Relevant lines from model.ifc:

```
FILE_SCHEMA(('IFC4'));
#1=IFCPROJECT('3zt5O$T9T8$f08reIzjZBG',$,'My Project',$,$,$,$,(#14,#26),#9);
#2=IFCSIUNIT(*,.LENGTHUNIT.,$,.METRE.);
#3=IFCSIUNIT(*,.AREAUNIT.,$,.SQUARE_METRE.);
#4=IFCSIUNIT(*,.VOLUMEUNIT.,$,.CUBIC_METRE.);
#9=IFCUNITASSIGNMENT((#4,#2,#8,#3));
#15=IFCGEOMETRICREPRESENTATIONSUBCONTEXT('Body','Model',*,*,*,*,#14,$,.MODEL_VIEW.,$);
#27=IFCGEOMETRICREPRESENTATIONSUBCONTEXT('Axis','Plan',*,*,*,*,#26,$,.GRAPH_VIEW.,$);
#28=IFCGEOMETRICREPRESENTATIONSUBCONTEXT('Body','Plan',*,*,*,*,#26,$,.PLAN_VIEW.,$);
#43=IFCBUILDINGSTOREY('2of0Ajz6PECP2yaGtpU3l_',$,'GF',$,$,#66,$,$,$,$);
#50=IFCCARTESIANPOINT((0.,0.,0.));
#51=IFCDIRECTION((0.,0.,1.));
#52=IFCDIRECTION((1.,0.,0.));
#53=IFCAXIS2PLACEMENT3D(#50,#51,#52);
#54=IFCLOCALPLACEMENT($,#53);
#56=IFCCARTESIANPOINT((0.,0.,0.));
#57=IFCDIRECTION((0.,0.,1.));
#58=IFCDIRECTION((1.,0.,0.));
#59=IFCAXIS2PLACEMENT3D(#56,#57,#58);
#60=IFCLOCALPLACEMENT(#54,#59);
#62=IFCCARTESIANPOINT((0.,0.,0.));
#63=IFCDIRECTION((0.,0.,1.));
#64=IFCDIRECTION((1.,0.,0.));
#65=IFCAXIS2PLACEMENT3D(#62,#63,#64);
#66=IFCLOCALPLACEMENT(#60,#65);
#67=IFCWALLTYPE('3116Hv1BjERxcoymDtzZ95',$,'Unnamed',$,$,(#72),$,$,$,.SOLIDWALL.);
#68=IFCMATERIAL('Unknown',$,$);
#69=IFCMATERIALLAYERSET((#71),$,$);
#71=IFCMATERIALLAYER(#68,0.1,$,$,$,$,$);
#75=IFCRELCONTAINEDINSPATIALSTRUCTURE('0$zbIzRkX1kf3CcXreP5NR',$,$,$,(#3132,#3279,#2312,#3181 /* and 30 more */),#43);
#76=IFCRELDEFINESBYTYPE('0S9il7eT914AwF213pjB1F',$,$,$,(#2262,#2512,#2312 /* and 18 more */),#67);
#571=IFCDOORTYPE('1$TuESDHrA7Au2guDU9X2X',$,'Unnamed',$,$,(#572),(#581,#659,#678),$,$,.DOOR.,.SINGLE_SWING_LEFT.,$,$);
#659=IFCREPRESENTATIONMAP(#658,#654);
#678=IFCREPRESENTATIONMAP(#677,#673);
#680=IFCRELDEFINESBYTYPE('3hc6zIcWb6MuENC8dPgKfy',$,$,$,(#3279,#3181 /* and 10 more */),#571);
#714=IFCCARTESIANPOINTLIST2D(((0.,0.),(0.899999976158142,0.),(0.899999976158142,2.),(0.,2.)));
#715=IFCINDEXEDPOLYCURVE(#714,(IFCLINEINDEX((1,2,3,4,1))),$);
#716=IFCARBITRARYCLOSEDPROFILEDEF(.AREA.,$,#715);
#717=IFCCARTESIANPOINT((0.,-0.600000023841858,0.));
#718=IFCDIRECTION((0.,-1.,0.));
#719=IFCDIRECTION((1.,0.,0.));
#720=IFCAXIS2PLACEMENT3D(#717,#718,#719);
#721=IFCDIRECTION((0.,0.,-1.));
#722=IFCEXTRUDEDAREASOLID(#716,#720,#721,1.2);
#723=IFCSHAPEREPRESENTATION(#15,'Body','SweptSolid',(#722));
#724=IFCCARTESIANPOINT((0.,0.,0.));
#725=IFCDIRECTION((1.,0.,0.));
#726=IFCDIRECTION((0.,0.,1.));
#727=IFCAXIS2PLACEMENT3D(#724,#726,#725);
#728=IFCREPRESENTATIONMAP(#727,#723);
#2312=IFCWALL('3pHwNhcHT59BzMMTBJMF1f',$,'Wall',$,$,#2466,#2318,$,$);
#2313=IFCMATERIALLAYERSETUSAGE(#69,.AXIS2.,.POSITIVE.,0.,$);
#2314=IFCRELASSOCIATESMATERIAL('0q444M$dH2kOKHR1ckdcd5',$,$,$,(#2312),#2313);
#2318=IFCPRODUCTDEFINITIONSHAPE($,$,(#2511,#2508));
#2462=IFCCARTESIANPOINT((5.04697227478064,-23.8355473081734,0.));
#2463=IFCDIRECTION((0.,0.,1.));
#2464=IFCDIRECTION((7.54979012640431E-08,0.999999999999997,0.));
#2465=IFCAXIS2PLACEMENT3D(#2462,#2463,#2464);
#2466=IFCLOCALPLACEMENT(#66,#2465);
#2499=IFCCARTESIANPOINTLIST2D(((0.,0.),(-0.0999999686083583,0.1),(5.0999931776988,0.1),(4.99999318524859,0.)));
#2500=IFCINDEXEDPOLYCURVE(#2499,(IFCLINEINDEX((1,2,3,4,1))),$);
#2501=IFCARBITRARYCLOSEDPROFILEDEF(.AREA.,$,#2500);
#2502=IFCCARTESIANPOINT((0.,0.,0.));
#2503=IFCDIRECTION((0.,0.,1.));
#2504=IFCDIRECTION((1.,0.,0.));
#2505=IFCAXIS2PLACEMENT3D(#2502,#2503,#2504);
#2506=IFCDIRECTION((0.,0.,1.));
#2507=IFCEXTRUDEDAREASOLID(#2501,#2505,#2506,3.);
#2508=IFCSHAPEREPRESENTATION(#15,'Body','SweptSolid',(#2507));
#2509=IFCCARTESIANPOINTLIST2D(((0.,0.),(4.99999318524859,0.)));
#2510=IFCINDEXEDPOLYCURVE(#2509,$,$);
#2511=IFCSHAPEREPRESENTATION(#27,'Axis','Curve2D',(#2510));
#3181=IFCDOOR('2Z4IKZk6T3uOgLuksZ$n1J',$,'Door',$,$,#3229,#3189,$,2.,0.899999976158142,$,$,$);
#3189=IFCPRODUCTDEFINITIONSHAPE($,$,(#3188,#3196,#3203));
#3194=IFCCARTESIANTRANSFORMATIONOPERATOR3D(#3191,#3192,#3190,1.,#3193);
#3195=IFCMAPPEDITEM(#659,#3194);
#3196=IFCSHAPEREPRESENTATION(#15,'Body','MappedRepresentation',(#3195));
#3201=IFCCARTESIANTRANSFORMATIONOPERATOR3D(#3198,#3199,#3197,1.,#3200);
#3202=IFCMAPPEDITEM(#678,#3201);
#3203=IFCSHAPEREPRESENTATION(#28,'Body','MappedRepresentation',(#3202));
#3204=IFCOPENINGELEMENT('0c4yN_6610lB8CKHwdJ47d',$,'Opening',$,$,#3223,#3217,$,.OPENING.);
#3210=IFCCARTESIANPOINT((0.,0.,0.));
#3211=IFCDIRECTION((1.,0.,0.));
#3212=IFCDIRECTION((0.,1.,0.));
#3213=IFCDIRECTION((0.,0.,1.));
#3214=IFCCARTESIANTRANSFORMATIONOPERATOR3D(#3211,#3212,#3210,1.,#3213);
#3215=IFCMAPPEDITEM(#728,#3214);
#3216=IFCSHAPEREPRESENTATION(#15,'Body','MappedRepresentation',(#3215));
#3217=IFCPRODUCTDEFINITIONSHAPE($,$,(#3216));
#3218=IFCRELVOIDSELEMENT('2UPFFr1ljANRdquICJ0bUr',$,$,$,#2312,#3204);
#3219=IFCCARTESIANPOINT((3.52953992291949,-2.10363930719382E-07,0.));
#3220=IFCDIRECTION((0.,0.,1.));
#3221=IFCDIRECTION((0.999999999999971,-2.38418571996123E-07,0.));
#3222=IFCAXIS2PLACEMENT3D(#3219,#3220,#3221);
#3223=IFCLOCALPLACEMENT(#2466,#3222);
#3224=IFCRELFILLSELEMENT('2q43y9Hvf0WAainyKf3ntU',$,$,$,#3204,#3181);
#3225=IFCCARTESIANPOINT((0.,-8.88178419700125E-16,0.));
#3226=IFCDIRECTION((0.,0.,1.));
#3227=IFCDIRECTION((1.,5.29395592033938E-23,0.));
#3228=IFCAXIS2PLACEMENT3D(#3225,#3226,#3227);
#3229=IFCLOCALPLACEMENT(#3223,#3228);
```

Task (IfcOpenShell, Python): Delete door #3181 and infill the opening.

```python
import ifcopenshell
import ifcopenshell.api.feature
import ifcopenshell.api.root
import ifcopenshell.geom
import ifcopenshell.util.shape

model = ifcopenshell.open("model.ifc")
settings = ifcopenshell.geom.settings()


def volume(element):
    """Net volume in cubic metres, openings subtracted."""
    shape = ifcopenshell.geom.create_shape(settings, element)
    return ifcopenshell.util.shape.get_volume(shape.geometry)


door = model.by_guid("2Z4IKZk6T3uOgLuksZ$n1J")
opening = door.FillsVoids[0].RelatingOpeningElement
wall = opening.VoidsElements[0].RelatingBuildingElement
before = volume(wall)

ifcopenshell.api.root.remove_product(model, product=door)
ifcopenshell.api.feature.remove_feature(model, feature=opening)

after = volume(wall)

print(f"wall volume {before:.3f} -> {after:.3f} m3")

model.write("model_updated.ifc")
```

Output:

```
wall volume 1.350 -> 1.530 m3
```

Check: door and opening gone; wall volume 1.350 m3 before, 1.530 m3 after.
